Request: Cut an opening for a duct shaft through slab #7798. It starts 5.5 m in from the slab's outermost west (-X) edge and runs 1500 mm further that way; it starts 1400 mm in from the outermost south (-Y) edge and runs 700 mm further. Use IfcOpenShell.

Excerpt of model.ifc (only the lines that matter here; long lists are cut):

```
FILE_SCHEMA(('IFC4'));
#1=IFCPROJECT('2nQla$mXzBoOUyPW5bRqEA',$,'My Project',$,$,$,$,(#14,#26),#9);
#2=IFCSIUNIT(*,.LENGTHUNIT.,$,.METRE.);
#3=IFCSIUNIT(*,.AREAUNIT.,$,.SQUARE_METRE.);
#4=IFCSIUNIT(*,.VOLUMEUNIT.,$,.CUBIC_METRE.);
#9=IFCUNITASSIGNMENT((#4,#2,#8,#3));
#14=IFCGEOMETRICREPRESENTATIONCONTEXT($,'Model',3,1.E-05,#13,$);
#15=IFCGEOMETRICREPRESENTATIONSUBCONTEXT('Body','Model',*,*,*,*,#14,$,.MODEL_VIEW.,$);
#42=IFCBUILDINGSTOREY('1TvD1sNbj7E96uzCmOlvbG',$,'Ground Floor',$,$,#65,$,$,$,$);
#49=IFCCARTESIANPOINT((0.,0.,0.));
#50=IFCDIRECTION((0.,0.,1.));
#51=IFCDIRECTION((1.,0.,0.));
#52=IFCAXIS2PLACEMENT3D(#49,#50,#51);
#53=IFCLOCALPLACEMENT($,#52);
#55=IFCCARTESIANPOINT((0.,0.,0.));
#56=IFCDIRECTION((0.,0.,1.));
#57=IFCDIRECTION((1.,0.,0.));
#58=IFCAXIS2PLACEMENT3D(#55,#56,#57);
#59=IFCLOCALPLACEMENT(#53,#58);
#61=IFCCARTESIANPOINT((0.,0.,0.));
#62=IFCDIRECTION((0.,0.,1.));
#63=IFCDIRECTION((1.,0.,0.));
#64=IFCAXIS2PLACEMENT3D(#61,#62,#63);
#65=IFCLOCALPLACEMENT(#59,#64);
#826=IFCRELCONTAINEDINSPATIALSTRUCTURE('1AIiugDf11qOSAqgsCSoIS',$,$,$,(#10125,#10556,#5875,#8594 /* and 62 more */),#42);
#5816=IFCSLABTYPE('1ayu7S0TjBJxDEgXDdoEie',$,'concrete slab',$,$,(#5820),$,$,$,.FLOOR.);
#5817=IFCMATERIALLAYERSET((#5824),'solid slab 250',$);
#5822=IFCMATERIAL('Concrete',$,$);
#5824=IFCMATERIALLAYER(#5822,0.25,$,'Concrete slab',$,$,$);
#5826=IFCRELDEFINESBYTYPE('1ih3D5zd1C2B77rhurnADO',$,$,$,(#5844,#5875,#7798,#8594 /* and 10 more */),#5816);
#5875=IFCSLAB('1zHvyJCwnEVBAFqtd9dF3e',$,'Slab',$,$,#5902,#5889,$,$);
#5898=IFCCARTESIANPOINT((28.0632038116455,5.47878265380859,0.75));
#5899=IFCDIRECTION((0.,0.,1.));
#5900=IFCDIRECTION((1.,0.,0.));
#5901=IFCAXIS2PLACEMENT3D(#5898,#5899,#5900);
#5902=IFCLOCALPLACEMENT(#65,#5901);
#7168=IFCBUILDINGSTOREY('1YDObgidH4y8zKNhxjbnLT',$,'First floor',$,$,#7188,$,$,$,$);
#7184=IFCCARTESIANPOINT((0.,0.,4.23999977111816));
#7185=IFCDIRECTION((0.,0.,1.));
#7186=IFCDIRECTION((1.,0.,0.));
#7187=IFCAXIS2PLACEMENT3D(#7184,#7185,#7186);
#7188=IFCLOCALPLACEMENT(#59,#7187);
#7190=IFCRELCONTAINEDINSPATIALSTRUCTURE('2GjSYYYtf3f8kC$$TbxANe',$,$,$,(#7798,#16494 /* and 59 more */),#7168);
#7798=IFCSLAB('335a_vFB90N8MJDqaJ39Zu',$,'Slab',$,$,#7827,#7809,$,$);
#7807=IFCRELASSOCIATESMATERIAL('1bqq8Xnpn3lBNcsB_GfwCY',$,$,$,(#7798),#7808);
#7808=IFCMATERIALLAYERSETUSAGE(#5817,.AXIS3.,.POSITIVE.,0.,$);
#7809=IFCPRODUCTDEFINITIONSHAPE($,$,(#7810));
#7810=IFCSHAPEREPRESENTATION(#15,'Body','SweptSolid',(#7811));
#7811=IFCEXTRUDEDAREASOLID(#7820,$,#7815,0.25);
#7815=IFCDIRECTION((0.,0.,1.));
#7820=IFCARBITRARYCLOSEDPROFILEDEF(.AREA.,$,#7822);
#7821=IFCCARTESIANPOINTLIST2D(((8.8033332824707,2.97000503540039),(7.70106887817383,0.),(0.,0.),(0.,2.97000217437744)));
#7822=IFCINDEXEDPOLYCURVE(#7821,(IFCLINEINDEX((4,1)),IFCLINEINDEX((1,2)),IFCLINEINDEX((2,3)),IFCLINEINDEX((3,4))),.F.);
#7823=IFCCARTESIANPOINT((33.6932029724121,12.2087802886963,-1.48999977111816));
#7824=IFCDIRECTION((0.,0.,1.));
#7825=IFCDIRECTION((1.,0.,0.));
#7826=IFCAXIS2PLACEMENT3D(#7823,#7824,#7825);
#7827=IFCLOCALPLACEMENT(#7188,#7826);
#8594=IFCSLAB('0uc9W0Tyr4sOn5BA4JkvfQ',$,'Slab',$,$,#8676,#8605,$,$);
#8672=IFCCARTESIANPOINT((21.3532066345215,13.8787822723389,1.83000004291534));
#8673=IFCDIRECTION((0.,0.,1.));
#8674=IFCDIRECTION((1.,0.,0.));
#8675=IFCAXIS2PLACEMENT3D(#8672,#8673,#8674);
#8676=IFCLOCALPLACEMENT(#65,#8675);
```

```python
import numpy as np
import ifcopenshell
import ifcopenshell.api.feature
import ifcopenshell.api.geometry
import ifcopenshell.api.root
import ifcopenshell.geom
import ifcopenshell.util.placement
import ifcopenshell.util.representation
import ifcopenshell.util.shape
import ifcopenshell.util.unit

model = ifcopenshell.open("model.ifc")
unit_scale = ifcopenshell.util.unit.calculate_unit_scale(model)
settings = ifcopenshell.geom.settings()


def volume(element):
    """Net volume in cubic metres, openings subtracted."""
    shape = ifcopenshell.geom.create_shape(settings, element)
    return ifcopenshell.util.shape.get_volume(shape.geometry)


slab = model.by_guid("335a_vFB90N8MJDqaJ39Zu")
before = volume(slab)

# Extent in the slab's own axes, in metres. The edges named are its -X and -Y sides.
slab_shape = ifcopenshell.geom.create_shape(settings, slab)
vertices = ifcopenshell.util.shape.get_vertices(slab_shape.geometry)
x_min, y_min, bottom = vertices.min(axis=0)
top = vertices[:, 2].max()

opening = ifcopenshell.api.root.create_entity(model, ifc_class="IfcOpeningElement", name="Duct shaft opening", predefined_type="OPENING")
context = ifcopenshell.util.representation.get_context(model, "Model", "Body", "MODEL_VIEW")
width, depth = 1.5, 0.7
outline = [(0.0, 0.0), (width, 0.0), (width, depth), (0.0, depth), (0.0, 0.0)]
# Overshoot both faces by 50 mm so the cut is clean.
shape = ifcopenshell.api.geometry.add_slab_representation(
    model, context=context, depth=top - bottom + 0.1, polyline=outline
)
ifcopenshell.api.geometry.assign_representation(model, product=opening, representation=shape)

matrix = ifcopenshell.util.placement.get_local_placement(slab.ObjectPlacement)
matrix[:, 3] = matrix @ np.append(np.array([x_min + 5.5, y_min + 1.4, bottom - 0.05]) / unit_scale, 1.0)
ifcopenshell.api.geometry.edit_object_placement(model, product=opening, matrix=matrix, is_si=False)
ifcopenshell.api.feature.add_feature(model, feature=opening, element=slab)

after = volume(slab)

print(f"slab volume {before:.3f} -> {after:.3f} m3")

model.write("model_rev.ifc")
```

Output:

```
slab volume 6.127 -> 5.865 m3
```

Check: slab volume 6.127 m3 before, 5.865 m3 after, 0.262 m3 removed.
